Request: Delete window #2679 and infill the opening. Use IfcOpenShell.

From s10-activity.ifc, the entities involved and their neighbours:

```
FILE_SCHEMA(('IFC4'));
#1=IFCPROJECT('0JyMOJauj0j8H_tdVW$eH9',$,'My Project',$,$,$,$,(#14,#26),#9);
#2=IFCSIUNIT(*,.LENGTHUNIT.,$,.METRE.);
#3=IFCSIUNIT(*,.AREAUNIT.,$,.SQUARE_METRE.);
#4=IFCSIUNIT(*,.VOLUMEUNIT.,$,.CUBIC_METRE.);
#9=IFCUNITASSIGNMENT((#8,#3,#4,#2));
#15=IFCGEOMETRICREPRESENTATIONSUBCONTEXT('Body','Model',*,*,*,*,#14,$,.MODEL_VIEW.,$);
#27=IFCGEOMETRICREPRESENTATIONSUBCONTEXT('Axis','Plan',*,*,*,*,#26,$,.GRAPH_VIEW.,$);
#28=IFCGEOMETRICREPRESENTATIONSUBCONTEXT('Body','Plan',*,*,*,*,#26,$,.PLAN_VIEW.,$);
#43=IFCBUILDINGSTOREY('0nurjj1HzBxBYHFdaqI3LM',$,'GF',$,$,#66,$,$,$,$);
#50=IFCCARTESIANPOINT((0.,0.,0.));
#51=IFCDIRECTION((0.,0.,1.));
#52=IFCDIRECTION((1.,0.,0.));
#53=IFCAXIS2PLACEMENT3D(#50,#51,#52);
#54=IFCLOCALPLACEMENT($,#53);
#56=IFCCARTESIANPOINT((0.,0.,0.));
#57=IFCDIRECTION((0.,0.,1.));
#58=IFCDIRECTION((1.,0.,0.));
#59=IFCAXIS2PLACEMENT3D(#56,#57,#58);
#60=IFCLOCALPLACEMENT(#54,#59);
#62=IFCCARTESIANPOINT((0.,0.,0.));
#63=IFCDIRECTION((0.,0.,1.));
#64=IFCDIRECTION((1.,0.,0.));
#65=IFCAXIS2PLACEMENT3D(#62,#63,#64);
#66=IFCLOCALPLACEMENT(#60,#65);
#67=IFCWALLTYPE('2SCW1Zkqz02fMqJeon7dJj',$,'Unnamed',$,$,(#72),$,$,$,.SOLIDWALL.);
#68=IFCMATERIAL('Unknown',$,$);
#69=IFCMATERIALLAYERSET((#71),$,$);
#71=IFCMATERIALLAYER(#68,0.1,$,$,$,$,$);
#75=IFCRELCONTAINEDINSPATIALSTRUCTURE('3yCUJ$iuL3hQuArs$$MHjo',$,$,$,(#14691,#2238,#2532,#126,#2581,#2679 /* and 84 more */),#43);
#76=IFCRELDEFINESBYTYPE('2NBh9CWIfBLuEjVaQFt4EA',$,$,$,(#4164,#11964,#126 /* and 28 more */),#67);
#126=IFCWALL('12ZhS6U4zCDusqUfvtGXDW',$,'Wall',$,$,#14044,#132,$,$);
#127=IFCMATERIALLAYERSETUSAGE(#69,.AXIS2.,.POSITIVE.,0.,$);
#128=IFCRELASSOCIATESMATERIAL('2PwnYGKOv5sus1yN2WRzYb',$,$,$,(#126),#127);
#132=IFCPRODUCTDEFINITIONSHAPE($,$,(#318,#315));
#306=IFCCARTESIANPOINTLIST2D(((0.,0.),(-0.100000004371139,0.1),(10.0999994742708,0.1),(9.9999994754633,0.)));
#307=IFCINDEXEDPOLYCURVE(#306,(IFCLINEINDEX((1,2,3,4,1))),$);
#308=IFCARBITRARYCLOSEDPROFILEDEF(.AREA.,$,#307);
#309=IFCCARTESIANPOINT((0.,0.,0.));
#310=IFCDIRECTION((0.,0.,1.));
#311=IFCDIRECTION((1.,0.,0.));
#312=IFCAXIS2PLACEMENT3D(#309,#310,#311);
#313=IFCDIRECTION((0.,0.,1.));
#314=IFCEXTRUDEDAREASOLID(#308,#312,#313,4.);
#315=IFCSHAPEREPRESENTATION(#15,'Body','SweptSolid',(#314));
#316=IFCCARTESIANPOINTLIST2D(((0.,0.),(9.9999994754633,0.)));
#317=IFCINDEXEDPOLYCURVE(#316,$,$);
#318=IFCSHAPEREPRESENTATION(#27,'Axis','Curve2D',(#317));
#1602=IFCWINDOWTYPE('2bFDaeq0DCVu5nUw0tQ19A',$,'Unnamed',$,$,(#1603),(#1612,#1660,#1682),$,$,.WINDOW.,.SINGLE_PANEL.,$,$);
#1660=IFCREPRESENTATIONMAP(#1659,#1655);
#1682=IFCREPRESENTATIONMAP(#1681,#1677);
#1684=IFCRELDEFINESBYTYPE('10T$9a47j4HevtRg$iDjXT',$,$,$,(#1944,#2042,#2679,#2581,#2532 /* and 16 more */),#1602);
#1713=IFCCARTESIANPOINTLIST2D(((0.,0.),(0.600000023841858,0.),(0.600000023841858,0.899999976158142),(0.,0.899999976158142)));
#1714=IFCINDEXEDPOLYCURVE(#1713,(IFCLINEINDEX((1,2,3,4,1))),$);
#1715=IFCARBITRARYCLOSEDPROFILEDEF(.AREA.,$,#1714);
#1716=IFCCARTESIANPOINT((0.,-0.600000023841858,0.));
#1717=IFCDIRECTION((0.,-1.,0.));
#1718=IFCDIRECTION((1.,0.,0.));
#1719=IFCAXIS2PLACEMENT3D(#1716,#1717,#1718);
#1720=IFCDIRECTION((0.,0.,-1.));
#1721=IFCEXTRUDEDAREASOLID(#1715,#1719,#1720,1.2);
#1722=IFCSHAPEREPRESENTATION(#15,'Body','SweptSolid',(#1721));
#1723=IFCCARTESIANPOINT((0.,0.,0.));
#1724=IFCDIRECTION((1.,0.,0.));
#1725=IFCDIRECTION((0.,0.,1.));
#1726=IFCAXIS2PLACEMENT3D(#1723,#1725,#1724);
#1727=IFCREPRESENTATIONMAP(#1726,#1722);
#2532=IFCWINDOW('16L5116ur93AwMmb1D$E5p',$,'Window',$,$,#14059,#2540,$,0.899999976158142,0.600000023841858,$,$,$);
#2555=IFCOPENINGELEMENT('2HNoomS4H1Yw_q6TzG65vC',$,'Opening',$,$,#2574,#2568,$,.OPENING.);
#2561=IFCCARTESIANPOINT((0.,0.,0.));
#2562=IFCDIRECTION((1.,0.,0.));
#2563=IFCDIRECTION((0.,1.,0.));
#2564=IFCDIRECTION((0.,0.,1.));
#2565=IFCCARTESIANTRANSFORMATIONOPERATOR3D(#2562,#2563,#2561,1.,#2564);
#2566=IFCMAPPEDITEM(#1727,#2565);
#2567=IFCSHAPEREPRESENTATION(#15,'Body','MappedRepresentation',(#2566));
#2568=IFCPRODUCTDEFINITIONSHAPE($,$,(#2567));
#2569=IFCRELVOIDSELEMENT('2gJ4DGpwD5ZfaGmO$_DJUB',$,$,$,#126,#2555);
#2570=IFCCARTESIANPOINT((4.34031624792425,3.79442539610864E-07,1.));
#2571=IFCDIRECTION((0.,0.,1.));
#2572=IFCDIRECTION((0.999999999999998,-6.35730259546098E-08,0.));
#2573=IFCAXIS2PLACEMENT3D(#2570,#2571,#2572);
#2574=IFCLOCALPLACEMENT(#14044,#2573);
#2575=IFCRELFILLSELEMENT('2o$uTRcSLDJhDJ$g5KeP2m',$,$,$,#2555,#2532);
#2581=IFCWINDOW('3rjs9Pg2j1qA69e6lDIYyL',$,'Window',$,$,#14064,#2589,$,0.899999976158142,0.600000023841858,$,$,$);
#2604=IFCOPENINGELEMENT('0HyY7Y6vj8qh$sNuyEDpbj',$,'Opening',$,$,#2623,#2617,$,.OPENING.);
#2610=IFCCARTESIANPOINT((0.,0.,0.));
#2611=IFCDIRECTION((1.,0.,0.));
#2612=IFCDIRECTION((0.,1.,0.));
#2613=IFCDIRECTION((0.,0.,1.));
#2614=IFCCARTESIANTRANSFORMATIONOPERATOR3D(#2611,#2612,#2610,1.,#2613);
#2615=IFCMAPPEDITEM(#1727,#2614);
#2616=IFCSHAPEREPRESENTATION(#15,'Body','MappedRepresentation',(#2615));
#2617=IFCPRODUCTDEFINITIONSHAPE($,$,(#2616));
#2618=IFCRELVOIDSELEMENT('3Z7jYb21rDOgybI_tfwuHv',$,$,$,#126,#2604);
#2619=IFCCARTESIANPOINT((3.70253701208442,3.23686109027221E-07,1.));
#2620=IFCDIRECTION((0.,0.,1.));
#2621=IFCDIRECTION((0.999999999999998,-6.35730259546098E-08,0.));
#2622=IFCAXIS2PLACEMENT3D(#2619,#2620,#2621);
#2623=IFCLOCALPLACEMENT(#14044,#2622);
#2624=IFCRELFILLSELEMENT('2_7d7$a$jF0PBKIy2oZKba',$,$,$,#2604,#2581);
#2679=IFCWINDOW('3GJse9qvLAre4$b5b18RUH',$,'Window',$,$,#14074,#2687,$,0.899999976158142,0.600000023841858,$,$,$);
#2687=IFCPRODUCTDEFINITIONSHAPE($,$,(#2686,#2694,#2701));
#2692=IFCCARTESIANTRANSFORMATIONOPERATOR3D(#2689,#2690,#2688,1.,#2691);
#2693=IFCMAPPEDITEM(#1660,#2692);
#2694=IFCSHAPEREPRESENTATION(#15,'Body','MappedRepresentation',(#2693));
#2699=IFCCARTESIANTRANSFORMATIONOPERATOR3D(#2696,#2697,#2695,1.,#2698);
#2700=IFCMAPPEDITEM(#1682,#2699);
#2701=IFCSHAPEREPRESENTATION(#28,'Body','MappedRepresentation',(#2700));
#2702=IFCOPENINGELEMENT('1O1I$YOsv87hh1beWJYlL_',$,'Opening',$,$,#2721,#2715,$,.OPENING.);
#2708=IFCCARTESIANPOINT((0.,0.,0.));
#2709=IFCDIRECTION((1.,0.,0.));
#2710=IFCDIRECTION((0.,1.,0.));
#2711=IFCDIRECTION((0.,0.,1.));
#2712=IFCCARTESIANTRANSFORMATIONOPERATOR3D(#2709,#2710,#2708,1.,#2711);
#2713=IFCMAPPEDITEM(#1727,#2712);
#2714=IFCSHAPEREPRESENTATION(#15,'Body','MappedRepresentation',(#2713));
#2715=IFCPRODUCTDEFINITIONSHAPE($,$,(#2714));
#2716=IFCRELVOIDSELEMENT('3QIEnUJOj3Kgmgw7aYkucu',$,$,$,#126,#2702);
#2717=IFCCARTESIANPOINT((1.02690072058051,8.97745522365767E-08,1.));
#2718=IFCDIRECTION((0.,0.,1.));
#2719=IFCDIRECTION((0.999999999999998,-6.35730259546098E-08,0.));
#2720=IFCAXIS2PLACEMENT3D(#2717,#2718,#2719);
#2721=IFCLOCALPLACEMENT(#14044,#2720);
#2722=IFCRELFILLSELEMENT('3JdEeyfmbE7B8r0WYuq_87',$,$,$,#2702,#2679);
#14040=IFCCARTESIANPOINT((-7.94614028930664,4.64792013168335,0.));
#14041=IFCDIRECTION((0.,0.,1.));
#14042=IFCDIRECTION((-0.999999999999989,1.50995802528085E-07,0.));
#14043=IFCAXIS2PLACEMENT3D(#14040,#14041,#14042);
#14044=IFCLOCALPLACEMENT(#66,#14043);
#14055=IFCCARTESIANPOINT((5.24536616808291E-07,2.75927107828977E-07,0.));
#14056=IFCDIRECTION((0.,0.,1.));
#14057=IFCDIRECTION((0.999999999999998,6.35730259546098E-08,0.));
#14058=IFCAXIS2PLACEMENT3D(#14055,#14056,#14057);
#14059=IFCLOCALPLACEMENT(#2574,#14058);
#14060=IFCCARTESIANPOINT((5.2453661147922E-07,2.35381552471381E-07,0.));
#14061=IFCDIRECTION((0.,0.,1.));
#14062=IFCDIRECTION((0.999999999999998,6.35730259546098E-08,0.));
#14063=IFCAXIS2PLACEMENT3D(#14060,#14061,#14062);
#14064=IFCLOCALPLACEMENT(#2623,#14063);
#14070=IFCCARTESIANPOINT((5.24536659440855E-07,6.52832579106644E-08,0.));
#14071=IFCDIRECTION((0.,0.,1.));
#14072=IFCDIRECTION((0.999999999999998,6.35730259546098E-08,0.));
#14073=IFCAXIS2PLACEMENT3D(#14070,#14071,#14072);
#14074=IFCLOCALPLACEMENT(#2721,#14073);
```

```python
import ifcopenshell
import ifcopenshell.api.feature
import ifcopenshell.api.root
import ifcopenshell.geom
import ifcopenshell.util.shape

model = ifcopenshell.open("s10-activity.ifc")
settings = ifcopenshell.geom.settings()


def volume(element):
    """Net volume in cubic metres, openings subtracted."""
    shape = ifcopenshell.geom.create_shape(settings, element)
    return ifcopenshell.util.shape.get_volume(shape.geometry)


window = model.by_guid("3GJse9qvLAre4$b5b18RUH")
opening = window.FillsVoids[0].RelatingOpeningElement
wall = opening.VoidsElements[0].RelatingBuildingElement
before = volume(wall)

ifcopenshell.api.root.remove_product(model, product=window)
ifcopenshell.api.feature.remove_feature(model, feature=opening)

after = volume(wall)

print(f"wall volume {before:.3f} -> {after:.3f} m3")

model.write("s10-activity_rev.ifc")
```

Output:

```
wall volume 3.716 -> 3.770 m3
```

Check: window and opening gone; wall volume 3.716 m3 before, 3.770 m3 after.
